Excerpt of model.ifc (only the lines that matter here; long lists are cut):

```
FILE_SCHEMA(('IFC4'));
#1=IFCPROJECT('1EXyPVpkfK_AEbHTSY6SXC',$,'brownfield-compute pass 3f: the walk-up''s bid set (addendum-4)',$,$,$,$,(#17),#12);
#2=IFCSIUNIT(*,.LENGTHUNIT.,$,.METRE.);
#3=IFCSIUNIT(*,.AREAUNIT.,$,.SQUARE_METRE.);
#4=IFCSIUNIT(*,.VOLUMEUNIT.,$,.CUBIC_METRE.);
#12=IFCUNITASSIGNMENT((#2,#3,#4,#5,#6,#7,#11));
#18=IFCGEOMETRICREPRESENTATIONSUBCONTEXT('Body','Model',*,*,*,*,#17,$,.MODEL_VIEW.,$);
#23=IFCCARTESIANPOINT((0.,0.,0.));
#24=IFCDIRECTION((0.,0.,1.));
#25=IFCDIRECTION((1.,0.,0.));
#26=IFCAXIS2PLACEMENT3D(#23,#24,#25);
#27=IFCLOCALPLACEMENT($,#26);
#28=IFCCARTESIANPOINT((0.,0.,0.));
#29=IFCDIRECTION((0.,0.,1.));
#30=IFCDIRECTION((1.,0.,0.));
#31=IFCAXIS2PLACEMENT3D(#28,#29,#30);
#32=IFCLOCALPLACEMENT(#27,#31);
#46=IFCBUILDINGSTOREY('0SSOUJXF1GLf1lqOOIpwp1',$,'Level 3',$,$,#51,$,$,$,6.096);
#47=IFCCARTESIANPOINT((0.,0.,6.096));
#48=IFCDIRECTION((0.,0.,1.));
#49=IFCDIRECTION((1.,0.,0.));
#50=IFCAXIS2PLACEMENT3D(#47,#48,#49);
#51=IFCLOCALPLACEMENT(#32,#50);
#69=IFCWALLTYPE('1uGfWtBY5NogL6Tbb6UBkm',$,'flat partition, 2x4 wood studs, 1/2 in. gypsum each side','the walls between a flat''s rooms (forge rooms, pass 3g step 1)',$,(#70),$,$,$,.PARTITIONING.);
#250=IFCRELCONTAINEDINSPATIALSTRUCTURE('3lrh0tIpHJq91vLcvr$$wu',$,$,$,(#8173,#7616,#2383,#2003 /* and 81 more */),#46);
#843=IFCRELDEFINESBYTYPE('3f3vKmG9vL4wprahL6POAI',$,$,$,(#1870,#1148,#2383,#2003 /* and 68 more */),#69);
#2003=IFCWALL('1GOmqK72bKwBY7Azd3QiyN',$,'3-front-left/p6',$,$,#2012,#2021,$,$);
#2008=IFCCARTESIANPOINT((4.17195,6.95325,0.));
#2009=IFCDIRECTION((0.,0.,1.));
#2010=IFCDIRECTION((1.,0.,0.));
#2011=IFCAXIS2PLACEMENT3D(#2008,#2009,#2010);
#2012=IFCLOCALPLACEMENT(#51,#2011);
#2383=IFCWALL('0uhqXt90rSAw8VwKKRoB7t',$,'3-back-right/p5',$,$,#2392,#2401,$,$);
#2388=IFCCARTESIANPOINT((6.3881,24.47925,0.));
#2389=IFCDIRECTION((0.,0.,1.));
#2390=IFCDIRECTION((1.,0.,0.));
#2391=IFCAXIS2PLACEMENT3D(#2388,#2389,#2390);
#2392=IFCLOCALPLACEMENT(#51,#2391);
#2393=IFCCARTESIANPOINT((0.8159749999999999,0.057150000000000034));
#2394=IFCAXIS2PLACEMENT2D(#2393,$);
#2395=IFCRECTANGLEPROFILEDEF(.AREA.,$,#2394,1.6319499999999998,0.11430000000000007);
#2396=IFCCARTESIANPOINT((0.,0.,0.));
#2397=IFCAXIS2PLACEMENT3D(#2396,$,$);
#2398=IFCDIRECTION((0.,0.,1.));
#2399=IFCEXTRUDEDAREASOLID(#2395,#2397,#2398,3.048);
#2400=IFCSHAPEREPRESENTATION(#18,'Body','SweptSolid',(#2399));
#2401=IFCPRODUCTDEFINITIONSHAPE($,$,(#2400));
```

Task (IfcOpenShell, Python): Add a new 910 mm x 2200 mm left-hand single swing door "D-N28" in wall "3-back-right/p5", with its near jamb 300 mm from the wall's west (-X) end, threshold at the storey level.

```python
import numpy as np
import ifcopenshell
import ifcopenshell.api.feature
import ifcopenshell.api.geometry
import ifcopenshell.api.root
import ifcopenshell.api.spatial
import ifcopenshell.geom
import ifcopenshell.util.element
import ifcopenshell.util.placement
import ifcopenshell.util.representation
import ifcopenshell.util.shape
import ifcopenshell.util.unit

model = ifcopenshell.open("model.ifc")
unit_scale = ifcopenshell.util.unit.calculate_unit_scale(model)
settings = ifcopenshell.geom.settings()


def volume(element):
    """Net volume in cubic metres, openings subtracted."""
    shape = ifcopenshell.geom.create_shape(settings, element)
    return ifcopenshell.util.shape.get_volume(shape.geometry)


wall = model.by_id(2383)
storey = ifcopenshell.util.element.get_container(wall, ifc_class="IfcBuildingStorey")
context = ifcopenshell.util.representation.get_context(model, "Model", "Body", "MODEL_VIEW")
before = volume(wall)

width, height, from_end, sill = 0.91, 2.2, 0.3, 0.0  # metres

# The wall runs along its own X axis, and the end named is its -X end.
wall_shape = ifcopenshell.geom.create_shape(settings, wall)
x, y, z = ifcopenshell.util.shape.get_vertices(wall_shape.geometry).T
start = x.min() + from_end
face, thickness = float(y.min()), float(y.max() - y.min())
wall_matrix = ifcopenshell.util.placement.get_local_placement(wall.ObjectPlacement)
level = ifcopenshell.util.placement.get_local_placement(storey.ObjectPlacement)[2, 3]


def in_wall(x, y):
    """Placement at x, y metres in the wall's axes, at sill height."""
    matrix = wall_matrix.copy()
    matrix[:, 3] = wall_matrix @ np.array([x / unit_scale, y / unit_scale, 0.0, 1.0])
    matrix[2, 3] = level + sill / unit_scale
    return matrix


# Opening: a box that overshoots both wall faces by 50 mm.
opening = ifcopenshell.api.root.create_entity(model, ifc_class="IfcOpeningElement", predefined_type="OPENING")
box = ifcopenshell.api.geometry.add_wall_representation(
    model, context=context, length=width, height=height, thickness=thickness + 0.1
)
ifcopenshell.api.geometry.assign_representation(model, product=opening, representation=box)
ifcopenshell.api.geometry.edit_object_placement(model, product=opening, matrix=in_wall(start, face - 0.05), is_si=False)
ifcopenshell.api.feature.add_feature(model, feature=opening, element=wall)

door = ifcopenshell.api.root.create_entity(model, ifc_class="IfcDoor", name="D-N28", predefined_type="DOOR")
door.OverallWidth, door.OverallHeight = width / unit_scale, height / unit_scale
door.OperationType = "SINGLE_SWING_LEFT"
body = ifcopenshell.api.geometry.add_door_representation(
    model,
    context=context,
    overall_width=door.OverallWidth,
    overall_height=door.OverallHeight,
    operation_type="SINGLE_SWING_LEFT",
    lining_properties={"LiningDepth": thickness / unit_scale, "ThresholdDepth": thickness / unit_scale},
)
ifcopenshell.api.geometry.assign_representation(model, product=door, representation=body)
ifcopenshell.api.spatial.assign_container(model, products=[door], relating_structure=storey)
ifcopenshell.api.feature.add_filling(model, opening=opening, element=door)

# The lining spans the wall, so the door starts at the wall face.
ifcopenshell.api.geometry.edit_object_placement(model, product=door, matrix=in_wall(start, face), is_si=False)

after = volume(wall)

print(f"wall volume {before:.3f} -> {after:.3f} m3")

model.write("model_edited.ifc")
```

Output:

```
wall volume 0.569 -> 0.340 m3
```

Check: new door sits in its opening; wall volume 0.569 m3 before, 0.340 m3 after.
